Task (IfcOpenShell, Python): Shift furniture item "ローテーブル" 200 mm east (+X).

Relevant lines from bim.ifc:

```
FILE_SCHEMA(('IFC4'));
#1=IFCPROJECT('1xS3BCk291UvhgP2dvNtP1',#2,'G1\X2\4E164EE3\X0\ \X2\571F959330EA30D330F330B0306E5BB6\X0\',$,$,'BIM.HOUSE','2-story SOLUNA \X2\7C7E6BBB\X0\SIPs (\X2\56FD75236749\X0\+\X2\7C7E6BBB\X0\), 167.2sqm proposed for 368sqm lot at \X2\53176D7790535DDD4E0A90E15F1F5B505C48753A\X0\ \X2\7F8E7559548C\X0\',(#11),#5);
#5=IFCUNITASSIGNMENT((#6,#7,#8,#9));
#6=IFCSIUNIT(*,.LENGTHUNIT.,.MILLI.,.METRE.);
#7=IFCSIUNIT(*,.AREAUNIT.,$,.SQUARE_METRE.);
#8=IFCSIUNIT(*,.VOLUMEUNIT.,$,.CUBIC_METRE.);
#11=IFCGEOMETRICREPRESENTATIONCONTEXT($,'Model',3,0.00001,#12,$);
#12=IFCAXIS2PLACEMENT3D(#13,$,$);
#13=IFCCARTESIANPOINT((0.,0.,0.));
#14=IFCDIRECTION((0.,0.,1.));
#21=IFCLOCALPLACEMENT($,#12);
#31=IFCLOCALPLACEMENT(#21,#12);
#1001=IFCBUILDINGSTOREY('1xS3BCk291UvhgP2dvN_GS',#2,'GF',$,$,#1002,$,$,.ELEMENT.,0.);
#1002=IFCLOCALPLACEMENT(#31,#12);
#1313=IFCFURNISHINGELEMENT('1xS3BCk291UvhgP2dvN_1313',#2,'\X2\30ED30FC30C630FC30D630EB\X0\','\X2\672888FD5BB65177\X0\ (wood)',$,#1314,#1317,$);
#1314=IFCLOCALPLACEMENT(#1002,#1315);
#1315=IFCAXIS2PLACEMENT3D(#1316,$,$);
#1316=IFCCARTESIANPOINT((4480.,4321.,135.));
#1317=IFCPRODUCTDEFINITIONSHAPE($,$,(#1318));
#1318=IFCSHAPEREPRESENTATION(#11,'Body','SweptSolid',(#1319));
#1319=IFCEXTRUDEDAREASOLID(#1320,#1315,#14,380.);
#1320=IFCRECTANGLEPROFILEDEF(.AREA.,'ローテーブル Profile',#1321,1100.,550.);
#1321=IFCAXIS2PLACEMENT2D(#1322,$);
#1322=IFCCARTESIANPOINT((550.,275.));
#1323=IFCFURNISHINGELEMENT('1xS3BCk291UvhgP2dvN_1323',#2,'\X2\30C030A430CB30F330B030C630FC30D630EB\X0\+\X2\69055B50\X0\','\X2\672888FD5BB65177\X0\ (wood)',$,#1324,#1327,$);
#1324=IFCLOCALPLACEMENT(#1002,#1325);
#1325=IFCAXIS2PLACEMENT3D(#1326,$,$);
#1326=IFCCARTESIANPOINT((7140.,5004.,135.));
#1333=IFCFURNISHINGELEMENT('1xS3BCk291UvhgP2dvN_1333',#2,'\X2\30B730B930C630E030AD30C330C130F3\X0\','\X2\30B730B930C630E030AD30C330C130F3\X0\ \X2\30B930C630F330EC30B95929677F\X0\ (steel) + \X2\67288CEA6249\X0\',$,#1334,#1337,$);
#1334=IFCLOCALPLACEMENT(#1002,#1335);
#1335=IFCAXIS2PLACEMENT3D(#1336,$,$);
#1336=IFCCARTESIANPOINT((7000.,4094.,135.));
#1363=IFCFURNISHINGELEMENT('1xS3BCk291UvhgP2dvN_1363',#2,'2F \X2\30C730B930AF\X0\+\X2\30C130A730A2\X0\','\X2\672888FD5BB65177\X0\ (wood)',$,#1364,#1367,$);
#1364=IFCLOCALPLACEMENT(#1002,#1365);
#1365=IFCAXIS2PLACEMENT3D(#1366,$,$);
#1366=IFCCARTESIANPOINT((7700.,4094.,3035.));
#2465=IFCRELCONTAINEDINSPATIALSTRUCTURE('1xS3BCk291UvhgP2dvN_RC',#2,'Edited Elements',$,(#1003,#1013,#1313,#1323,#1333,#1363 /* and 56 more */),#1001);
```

```python
import ifcopenshell
import ifcopenshell.api.geometry
import ifcopenshell.util.placement
import ifcopenshell.util.unit

model = ifcopenshell.open("bim.ifc")
unit_scale = ifcopenshell.util.unit.calculate_unit_scale(model)

item = model.by_guid("1xS3BCk291UvhgP2dvN_1313")
matrix = ifcopenshell.util.placement.get_local_placement(item.ObjectPlacement)
matrix[0, 3] += 0.2 / unit_scale
ifcopenshell.api.geometry.edit_object_placement(model, product=item, matrix=matrix, is_si=False)

print(ifcopenshell.util.placement.get_local_placement(item.ObjectPlacement).round(3) + 0.0)

model.write("bim_updated.ifc")
```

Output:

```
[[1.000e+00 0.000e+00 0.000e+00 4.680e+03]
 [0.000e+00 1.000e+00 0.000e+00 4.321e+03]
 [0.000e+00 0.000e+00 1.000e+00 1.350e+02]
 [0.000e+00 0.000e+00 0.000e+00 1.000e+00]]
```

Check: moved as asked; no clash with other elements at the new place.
